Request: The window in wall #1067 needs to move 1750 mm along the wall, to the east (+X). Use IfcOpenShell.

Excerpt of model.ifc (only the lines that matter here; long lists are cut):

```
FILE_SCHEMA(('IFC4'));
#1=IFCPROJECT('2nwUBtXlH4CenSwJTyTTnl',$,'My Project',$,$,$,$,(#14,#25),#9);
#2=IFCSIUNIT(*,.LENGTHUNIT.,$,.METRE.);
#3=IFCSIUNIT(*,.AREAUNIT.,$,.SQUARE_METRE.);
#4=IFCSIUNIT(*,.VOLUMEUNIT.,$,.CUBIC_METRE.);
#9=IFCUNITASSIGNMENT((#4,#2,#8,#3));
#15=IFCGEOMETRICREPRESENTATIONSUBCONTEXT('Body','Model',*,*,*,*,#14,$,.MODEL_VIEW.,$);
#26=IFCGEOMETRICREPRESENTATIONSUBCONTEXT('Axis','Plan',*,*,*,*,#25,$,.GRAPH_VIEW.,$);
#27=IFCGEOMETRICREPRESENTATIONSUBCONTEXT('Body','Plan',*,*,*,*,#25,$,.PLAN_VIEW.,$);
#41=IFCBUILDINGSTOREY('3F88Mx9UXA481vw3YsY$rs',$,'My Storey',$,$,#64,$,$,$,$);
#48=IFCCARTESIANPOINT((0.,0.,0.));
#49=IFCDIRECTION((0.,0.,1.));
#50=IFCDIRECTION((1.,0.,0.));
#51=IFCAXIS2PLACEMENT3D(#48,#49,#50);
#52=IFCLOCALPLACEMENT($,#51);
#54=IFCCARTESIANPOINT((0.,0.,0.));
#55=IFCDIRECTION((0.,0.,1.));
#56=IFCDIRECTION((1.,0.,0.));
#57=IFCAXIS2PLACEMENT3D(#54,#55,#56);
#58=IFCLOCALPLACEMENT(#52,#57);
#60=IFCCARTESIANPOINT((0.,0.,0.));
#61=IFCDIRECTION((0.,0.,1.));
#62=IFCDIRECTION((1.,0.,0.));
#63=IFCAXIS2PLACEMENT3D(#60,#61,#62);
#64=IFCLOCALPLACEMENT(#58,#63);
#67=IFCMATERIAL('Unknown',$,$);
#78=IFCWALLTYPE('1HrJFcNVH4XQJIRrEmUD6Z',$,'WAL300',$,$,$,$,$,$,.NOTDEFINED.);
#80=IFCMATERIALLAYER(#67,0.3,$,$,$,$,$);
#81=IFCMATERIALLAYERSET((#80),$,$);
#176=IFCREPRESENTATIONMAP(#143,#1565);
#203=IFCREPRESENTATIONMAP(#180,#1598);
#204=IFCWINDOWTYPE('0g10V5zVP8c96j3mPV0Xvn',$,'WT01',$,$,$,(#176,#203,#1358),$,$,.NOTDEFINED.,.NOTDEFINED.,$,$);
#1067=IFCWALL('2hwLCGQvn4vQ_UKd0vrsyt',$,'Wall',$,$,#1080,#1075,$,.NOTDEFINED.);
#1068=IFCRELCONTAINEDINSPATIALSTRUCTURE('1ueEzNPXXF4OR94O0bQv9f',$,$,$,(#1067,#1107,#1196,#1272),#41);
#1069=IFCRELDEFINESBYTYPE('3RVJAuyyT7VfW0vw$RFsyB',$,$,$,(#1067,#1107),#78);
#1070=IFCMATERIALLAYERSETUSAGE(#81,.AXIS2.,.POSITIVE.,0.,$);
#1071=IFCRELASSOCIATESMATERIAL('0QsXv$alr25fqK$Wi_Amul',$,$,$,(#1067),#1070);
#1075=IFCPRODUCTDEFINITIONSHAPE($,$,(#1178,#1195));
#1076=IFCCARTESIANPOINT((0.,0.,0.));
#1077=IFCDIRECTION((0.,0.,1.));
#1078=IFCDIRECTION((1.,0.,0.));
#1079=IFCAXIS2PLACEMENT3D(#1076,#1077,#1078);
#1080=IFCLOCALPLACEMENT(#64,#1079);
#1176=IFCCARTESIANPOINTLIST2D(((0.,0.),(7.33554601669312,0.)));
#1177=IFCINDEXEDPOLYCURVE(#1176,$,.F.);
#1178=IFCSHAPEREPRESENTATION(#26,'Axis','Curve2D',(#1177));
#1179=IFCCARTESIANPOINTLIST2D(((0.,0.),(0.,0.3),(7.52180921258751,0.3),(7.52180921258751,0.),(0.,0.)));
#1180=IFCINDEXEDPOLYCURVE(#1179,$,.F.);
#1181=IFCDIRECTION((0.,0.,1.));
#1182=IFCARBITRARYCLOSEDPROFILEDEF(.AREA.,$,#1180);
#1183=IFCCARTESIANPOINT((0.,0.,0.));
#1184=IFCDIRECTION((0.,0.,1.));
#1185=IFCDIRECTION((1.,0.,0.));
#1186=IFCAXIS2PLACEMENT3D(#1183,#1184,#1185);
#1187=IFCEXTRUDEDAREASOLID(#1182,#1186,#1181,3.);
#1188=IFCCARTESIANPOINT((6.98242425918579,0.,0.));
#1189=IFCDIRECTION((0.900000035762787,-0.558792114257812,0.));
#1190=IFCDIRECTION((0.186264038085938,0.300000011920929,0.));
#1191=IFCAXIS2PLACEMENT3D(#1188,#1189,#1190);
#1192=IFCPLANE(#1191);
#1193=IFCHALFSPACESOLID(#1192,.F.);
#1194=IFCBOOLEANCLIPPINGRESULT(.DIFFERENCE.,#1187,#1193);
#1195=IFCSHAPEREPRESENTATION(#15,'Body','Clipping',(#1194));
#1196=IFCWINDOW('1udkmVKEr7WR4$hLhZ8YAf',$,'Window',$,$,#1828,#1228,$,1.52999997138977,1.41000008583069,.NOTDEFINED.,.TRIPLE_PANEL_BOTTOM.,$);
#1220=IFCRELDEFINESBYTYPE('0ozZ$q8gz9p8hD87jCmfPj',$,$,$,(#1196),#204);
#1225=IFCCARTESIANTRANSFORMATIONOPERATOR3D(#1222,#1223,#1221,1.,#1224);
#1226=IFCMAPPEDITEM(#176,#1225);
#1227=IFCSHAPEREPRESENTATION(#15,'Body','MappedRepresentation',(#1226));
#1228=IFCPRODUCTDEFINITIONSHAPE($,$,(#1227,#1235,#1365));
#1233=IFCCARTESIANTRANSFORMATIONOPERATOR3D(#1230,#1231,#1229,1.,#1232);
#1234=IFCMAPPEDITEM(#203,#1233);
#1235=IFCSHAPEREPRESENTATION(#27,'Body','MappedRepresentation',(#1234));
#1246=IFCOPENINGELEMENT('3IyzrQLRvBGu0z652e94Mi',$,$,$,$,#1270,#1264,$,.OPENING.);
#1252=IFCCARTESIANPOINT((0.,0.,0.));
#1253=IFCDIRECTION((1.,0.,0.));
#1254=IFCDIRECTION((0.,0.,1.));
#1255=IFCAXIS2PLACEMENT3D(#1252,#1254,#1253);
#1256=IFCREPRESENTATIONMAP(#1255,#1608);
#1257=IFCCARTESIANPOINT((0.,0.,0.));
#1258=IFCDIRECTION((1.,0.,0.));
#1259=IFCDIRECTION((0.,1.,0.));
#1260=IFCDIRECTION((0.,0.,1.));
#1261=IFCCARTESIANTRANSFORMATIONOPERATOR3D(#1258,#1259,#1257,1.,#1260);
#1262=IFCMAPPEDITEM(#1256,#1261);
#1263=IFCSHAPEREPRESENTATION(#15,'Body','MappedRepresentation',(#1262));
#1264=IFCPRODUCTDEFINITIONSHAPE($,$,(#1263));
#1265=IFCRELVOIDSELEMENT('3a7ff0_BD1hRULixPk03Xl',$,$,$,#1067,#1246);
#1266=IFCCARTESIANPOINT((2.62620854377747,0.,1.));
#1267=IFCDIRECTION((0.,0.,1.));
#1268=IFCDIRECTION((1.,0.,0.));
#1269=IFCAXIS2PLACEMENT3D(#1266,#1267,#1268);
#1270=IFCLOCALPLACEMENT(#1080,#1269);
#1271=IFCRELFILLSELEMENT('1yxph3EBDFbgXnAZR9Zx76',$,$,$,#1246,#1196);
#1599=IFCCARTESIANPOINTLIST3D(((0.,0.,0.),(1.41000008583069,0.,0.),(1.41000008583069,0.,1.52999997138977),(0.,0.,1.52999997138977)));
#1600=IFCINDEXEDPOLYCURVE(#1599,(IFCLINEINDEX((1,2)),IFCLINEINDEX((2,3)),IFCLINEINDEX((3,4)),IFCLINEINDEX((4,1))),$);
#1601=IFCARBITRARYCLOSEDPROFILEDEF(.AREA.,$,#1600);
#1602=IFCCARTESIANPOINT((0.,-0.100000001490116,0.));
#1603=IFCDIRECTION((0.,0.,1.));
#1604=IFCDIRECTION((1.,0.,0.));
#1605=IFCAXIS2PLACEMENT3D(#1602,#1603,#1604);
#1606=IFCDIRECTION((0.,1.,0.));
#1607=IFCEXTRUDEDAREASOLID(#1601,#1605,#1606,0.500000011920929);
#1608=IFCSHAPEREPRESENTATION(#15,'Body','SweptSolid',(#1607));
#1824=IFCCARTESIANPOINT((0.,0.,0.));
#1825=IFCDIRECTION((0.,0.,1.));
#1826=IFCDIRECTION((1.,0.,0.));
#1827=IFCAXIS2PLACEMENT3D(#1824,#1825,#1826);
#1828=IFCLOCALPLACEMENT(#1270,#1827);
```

```python
import ifcopenshell
import ifcopenshell.api.geometry
import ifcopenshell.util.placement
import ifcopenshell.util.unit

model = ifcopenshell.open("model.ifc")
unit_scale = ifcopenshell.util.unit.calculate_unit_scale(model)

window = model.by_id(1196)
opening = window.FillsVoids[0].RelatingOpeningElement
wall = opening.VoidsElements[0].RelatingBuildingElement

wall_matrix = ifcopenshell.util.placement.get_local_placement(wall.ObjectPlacement)
shift = wall_matrix[:3, 0] * 1.75 / unit_scale
before = ifcopenshell.util.placement.get_local_placement(window.ObjectPlacement)[:3, 3].copy()

# The window is placed relative to its opening, so it follows when the opening moves.
matrix = ifcopenshell.util.placement.get_local_placement(opening.ObjectPlacement)
matrix[:3, 3] += shift
ifcopenshell.api.geometry.edit_object_placement(
    model, product=opening, matrix=matrix, is_si=False, should_transform_children=True
)

after = ifcopenshell.util.placement.get_local_placement(window.ObjectPlacement)[:3, 3]
print("window moved by", (after - before).round(3) + 0.0)

model.write("model_edited.ifc")
```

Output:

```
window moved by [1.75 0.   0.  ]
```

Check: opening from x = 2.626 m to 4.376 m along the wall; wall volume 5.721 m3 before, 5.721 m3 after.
